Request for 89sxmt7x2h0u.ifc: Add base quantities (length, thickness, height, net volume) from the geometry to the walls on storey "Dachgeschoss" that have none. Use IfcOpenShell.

First a look at what the model holds.

```python
import ifcopenshell
import ifcopenshell.util.element
import ifcopenshell.util.unit

model = ifcopenshell.open("89sxmt7x2h0u.ifc")
print(model.schema)
for unit_type in ("LENGTHUNIT", "AREAUNIT", "VOLUMEUNIT"):
    print(unit_type, ifcopenshell.util.unit.calculate_unit_scale(model, unit_type))
storey = next(s for s in model.by_type("IfcBuildingStorey") if s.Name == "Dachgeschoss")
walls = [e for e in ifcopenshell.util.element.get_decomposition(storey) if e.is_a("IfcWall")]
for e in sorted(walls, key=lambda e: e.id()):
    print(e.id(), e.is_a(), e.Name, list(ifcopenshell.util.element.get_psets(e, qtos_only=True)), sep=" | ")
```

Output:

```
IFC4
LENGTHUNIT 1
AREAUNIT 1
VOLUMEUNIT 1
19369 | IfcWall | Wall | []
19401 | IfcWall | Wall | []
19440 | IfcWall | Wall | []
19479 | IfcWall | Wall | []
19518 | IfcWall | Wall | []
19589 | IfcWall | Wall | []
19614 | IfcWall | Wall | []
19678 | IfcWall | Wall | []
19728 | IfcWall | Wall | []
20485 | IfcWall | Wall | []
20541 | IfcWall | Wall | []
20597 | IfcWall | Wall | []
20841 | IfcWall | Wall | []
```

```python
import ifcopenshell
import ifcopenshell.api.pset
import ifcopenshell.geom
import ifcopenshell.util.element
import ifcopenshell.util.shape
import ifcopenshell.util.unit

model = ifcopenshell.open("89sxmt7x2h0u.ifc")
unit_scale = ifcopenshell.util.unit.calculate_unit_scale(model)
volume_scale = ifcopenshell.util.unit.calculate_unit_scale(model, "VOLUMEUNIT")
settings = ifcopenshell.geom.settings()

storey = next(s for s in model.by_type("IfcBuildingStorey") if s.Name == "Dachgeschoss")
walls = [e for e in ifcopenshell.util.element.get_decomposition(storey) if e.is_a("IfcWall")]

for e in sorted(walls, key=lambda e: e.id()):
    if ifcopenshell.util.element.get_psets(e, qtos_only=True, should_inherit=False):
        continue
    # Geometry comes back in metres, in the element's own axes.
    shape = ifcopenshell.geom.create_shape(settings, e)
    values = {
        "Length": ifcopenshell.util.shape.get_x(shape.geometry) / unit_scale,
        "Width": ifcopenshell.util.shape.get_y(shape.geometry) / unit_scale,
        "Height": ifcopenshell.util.shape.get_z(shape.geometry) / unit_scale,
        "NetVolume": ifcopenshell.util.shape.get_volume(shape.geometry) / volume_scale,
    }
    qto = ifcopenshell.api.pset.add_qto(model, product=e, name="Qto_WallBaseQuantities")
    ifcopenshell.api.pset.edit_qto(model, qto=qto, properties=values)
    print(e.id(), {k: round(v, 3) for k, v in values.items()})

model.write("89sxmt7x2h0u-out.ifc")
```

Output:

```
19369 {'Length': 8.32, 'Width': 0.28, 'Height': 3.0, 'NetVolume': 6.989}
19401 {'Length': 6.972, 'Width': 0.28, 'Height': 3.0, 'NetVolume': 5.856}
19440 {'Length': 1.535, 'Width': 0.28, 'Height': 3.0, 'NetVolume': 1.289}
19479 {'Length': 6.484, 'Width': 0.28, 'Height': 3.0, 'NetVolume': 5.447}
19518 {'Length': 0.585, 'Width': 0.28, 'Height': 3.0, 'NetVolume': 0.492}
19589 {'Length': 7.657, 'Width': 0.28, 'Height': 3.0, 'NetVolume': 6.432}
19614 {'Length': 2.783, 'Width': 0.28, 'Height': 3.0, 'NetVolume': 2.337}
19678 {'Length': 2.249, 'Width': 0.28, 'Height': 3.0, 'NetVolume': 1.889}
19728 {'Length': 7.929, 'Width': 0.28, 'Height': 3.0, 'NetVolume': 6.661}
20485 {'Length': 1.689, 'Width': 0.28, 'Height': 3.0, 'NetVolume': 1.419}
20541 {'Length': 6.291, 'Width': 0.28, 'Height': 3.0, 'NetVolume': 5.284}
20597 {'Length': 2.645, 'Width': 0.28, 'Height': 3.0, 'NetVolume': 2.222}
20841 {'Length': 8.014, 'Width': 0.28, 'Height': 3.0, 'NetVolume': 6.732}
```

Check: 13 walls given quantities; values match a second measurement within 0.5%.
